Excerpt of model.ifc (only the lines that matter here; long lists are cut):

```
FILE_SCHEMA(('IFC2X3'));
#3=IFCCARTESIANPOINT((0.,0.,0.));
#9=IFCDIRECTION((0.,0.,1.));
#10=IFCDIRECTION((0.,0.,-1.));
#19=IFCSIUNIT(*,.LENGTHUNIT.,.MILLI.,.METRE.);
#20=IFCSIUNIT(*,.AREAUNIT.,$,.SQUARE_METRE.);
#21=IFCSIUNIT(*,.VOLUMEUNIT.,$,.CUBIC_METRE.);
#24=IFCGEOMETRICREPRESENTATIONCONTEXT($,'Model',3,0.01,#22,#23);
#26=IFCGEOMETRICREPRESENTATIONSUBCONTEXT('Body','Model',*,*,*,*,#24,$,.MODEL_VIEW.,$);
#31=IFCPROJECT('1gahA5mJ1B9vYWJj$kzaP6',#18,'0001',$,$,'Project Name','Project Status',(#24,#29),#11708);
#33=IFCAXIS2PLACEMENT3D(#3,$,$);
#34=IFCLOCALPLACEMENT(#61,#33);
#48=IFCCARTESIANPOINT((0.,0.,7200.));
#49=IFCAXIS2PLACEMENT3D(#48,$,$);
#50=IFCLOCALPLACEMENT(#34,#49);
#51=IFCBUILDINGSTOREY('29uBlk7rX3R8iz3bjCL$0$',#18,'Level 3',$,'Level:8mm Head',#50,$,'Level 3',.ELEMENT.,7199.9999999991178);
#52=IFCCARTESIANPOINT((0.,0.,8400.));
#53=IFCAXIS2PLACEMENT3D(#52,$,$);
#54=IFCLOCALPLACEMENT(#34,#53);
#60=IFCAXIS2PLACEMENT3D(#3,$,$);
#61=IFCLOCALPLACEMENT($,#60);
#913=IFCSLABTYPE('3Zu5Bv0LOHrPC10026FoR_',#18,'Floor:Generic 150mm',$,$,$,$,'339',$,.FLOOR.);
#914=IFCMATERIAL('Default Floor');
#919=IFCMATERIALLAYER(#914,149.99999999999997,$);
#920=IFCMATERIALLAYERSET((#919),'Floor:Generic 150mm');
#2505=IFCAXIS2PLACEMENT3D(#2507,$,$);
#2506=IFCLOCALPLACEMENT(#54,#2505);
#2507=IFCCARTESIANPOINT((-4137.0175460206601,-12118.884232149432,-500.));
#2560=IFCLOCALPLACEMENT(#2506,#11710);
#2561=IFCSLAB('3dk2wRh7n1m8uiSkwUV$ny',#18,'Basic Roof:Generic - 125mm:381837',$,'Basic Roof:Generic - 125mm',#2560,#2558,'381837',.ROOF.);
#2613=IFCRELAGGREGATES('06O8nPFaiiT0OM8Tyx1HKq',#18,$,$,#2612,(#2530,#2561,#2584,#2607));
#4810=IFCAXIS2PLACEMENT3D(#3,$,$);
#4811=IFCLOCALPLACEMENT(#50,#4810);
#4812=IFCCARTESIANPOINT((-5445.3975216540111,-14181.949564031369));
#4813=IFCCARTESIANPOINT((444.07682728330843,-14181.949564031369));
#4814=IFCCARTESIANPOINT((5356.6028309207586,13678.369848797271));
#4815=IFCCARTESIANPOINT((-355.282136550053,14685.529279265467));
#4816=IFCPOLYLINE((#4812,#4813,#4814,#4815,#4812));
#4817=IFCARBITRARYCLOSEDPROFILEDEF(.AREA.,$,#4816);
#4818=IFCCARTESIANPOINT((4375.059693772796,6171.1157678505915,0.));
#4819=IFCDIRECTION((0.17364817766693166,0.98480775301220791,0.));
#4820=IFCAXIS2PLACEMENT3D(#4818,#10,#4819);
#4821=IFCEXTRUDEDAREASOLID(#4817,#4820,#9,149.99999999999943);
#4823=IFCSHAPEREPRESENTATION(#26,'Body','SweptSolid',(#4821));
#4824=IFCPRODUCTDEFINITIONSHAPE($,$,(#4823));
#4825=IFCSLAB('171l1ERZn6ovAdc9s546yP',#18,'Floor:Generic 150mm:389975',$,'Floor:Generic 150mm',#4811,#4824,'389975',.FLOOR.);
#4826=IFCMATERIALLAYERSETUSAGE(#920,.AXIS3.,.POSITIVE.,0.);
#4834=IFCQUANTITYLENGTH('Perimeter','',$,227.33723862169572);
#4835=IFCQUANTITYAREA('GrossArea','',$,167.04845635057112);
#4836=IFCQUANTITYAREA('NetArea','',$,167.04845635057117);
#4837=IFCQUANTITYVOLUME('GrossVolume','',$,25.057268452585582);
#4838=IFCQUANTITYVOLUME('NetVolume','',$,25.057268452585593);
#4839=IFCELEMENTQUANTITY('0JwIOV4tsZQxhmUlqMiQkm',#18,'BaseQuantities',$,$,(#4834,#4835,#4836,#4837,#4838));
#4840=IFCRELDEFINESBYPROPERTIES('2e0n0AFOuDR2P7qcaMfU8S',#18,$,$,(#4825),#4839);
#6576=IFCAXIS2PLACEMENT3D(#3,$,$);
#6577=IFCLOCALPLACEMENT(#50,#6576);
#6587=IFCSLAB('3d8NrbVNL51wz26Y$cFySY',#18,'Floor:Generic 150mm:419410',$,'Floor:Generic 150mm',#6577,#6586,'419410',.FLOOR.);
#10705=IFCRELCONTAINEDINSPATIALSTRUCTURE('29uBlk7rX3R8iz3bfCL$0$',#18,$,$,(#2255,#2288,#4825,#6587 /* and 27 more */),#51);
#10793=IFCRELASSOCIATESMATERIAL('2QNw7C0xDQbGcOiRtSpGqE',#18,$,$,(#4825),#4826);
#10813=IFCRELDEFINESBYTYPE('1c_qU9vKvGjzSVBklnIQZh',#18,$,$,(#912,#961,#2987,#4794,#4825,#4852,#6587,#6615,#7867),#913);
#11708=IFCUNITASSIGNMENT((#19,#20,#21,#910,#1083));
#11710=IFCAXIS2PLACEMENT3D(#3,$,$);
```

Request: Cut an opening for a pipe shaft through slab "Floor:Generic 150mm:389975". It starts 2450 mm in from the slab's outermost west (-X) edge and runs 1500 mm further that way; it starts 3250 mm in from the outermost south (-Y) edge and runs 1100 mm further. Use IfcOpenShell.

```python
import numpy as np
import ifcopenshell
import ifcopenshell.api.feature
import ifcopenshell.api.geometry
import ifcopenshell.api.pset
import ifcopenshell.api.root
import ifcopenshell.geom
import ifcopenshell.util.element
import ifcopenshell.util.placement
import ifcopenshell.util.representation
import ifcopenshell.util.shape
import ifcopenshell.util.unit

model = ifcopenshell.open("model.ifc")
unit_scale = ifcopenshell.util.unit.calculate_unit_scale(model)
area_scale = ifcopenshell.util.unit.calculate_unit_scale(model, "AREAUNIT")
volume_scale = ifcopenshell.util.unit.calculate_unit_scale(model, "VOLUMEUNIT")
settings = ifcopenshell.geom.settings()


def volume(element):
    """Net volume in cubic metres, openings subtracted."""
    shape = ifcopenshell.geom.create_shape(settings, element)
    return ifcopenshell.util.shape.get_volume(shape.geometry)


slab = model.by_id(4825)
before = volume(slab)

# Extent in the slab's own axes, in metres. The edges named are its -X and -Y sides.
slab_shape = ifcopenshell.geom.create_shape(settings, slab)
vertices = ifcopenshell.util.shape.get_vertices(slab_shape.geometry)
x_min, y_min, bottom = vertices.min(axis=0)
top = vertices[:, 2].max()

opening = ifcopenshell.api.root.create_entity(model, ifc_class="IfcOpeningElement", name="Pipe shaft opening")
context = ifcopenshell.util.representation.get_context(model, "Model", "Body", "MODEL_VIEW")
width, depth = 1.5, 1.1
outline = [(0.0, 0.0), (width, 0.0), (width, depth), (0.0, depth), (0.0, 0.0)]
# Overshoot both faces by 50 mm so the cut is clean.
shape = ifcopenshell.api.geometry.add_slab_representation(
    model, context=context, depth=top - bottom + 0.1, polyline=outline
)
ifcopenshell.api.geometry.assign_representation(model, product=opening, representation=shape)

matrix = ifcopenshell.util.placement.get_local_placement(slab.ObjectPlacement)
matrix[:, 3] = matrix @ np.append(np.array([x_min + 2.45, y_min + 3.25, bottom - 0.05]) / unit_scale, 1.0)
ifcopenshell.api.geometry.edit_object_placement(model, product=opening, matrix=matrix, is_si=False)
ifcopenshell.api.feature.add_feature(model, feature=opening, element=slab)

after = volume(slab)

# Update the slab's stored quantities.
qto = model.by_id(ifcopenshell.util.element.get_pset(slab, "BaseQuantities", should_inherit=False)["id"])
ifcopenshell.api.pset.edit_qto(model, qto=qto, properties={
    "NetArea": after / (top - bottom) / area_scale,
    "NetVolume": after / volume_scale,
})

print(f"slab volume {before:.3f} -> {after:.3f} m3")

model.write("model-out.ifc")
```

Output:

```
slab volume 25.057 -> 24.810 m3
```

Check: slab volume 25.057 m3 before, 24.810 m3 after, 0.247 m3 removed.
